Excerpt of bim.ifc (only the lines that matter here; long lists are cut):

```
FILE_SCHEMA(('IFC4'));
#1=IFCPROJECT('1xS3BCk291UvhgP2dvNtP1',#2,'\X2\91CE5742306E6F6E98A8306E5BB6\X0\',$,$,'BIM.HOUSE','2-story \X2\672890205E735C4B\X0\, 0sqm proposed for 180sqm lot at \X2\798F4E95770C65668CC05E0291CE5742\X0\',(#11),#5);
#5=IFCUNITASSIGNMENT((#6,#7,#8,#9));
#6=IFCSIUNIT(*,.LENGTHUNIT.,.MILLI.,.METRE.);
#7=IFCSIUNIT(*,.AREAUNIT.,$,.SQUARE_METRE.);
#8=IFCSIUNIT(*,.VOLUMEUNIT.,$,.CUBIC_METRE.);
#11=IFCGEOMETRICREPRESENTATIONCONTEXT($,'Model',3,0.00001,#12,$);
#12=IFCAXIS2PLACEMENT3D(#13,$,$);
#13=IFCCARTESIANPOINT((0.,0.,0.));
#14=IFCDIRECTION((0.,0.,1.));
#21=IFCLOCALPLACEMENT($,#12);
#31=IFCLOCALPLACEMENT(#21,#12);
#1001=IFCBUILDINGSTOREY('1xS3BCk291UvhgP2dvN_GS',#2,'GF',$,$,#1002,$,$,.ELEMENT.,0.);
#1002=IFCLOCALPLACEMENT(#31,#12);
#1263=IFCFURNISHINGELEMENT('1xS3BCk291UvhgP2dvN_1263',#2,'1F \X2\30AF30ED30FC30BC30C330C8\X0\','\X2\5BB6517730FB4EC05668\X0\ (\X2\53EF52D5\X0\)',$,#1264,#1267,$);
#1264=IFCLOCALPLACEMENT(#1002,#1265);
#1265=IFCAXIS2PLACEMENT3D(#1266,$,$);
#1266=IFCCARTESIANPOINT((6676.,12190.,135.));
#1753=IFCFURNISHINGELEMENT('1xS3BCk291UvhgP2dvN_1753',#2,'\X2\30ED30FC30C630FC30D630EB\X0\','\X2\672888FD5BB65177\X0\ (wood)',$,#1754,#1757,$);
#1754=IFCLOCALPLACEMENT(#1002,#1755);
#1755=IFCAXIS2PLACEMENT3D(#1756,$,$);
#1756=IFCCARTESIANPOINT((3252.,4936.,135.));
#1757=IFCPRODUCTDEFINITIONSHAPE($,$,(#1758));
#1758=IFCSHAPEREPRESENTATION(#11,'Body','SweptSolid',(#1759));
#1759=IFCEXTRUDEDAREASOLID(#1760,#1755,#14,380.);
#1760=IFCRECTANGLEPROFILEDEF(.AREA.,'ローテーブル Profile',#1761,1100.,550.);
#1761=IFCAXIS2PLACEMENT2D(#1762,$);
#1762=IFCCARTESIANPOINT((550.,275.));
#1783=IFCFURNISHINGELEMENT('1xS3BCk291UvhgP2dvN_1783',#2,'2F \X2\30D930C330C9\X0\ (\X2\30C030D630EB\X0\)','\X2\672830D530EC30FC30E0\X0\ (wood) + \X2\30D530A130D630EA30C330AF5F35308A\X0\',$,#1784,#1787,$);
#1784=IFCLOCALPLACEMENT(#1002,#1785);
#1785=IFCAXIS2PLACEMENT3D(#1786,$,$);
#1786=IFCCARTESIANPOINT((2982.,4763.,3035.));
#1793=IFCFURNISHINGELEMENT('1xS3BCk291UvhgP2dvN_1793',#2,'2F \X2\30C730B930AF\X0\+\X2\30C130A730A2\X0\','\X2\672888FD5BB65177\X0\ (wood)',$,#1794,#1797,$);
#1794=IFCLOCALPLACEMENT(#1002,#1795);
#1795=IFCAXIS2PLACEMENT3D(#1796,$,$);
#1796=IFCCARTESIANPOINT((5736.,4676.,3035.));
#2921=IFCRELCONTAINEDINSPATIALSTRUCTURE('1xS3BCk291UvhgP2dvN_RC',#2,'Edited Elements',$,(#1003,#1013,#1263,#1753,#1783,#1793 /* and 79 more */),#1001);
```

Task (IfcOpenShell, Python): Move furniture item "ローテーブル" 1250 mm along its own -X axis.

```python
import ifcopenshell
import ifcopenshell.api.geometry
import ifcopenshell.util.placement
import ifcopenshell.util.unit

model = ifcopenshell.open("bim.ifc")
unit_scale = ifcopenshell.util.unit.calculate_unit_scale(model)

item = model.by_id(1753)
matrix = ifcopenshell.util.placement.get_local_placement(item.ObjectPlacement)
matrix[:3, 3] -= matrix[:3, 0] * 1.25 / unit_scale
ifcopenshell.api.geometry.edit_object_placement(model, product=item, matrix=matrix, is_si=False)

print(ifcopenshell.util.placement.get_local_placement(item.ObjectPlacement).round(3) + 0.0)

model.write("bim-out.ifc")
```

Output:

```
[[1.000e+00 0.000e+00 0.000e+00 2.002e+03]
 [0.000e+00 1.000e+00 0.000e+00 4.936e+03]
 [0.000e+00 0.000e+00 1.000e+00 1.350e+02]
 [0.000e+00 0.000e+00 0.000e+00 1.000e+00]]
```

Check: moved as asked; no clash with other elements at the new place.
